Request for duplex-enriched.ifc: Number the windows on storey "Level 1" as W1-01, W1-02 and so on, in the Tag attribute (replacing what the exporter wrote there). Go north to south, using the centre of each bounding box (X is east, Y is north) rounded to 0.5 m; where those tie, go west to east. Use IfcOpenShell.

First a look at what the model holds.

```python
import ifcopenshell
import ifcopenshell.util.element
import ifcopenshell.util.placement

model = ifcopenshell.open("duplex-enriched.ifc")
print(model.schema)
storey = next(s for s in model.by_type("IfcBuildingStorey") if s.Name == "Level 1")
windows = [e for e in ifcopenshell.util.element.get_decomposition(storey) if e.is_a("IfcWindow")]
for e in sorted(windows, key=lambda e: e.id()):
    origin = ifcopenshell.util.placement.get_local_placement(e.ObjectPlacement)[:3, 3]
    print(e.id(), e.Tag, e.Name, origin.round(2) + 0.0, sep=" | ")
```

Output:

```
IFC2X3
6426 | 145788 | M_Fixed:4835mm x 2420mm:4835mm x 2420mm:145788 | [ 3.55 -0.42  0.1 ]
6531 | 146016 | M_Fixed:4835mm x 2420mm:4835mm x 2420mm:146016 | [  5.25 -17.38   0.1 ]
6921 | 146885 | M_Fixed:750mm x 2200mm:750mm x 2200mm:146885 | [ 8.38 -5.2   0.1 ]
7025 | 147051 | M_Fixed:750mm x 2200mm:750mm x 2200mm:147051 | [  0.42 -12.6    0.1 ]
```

```python
import ifcopenshell
import ifcopenshell.geom
import ifcopenshell.util.element
import ifcopenshell.util.shape

model = ifcopenshell.open("duplex-enriched.ifc")
settings = ifcopenshell.geom.settings()
settings.set("use-world-coords", True)


def centre(element):
    shape = ifcopenshell.geom.create_shape(settings, element)
    return ifcopenshell.util.shape.get_bbox_centroid(shape.geometry)


storey = next(s for s in model.by_type("IfcBuildingStorey") if s.Name == "Level 1")
windows = [e for e in ifcopenshell.util.element.get_decomposition(storey) if e.is_a("IfcWindow")]

# Insertion points can sit at a corner or the storey origin, so sort by the geometry (in metres).
centres = {e: centre(e) for e in windows}
windows.sort(key=lambda e: (-round(centres[e][1] / 0.5), centres[e][0]))

for i, e in enumerate(windows, start=1):
    number = f"W1-{i:02d}"
    e.Tag = number
    print(e.id(), number)

model.write("duplex-enriched_rev.ifc")
```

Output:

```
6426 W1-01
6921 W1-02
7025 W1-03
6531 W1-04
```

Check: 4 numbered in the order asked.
